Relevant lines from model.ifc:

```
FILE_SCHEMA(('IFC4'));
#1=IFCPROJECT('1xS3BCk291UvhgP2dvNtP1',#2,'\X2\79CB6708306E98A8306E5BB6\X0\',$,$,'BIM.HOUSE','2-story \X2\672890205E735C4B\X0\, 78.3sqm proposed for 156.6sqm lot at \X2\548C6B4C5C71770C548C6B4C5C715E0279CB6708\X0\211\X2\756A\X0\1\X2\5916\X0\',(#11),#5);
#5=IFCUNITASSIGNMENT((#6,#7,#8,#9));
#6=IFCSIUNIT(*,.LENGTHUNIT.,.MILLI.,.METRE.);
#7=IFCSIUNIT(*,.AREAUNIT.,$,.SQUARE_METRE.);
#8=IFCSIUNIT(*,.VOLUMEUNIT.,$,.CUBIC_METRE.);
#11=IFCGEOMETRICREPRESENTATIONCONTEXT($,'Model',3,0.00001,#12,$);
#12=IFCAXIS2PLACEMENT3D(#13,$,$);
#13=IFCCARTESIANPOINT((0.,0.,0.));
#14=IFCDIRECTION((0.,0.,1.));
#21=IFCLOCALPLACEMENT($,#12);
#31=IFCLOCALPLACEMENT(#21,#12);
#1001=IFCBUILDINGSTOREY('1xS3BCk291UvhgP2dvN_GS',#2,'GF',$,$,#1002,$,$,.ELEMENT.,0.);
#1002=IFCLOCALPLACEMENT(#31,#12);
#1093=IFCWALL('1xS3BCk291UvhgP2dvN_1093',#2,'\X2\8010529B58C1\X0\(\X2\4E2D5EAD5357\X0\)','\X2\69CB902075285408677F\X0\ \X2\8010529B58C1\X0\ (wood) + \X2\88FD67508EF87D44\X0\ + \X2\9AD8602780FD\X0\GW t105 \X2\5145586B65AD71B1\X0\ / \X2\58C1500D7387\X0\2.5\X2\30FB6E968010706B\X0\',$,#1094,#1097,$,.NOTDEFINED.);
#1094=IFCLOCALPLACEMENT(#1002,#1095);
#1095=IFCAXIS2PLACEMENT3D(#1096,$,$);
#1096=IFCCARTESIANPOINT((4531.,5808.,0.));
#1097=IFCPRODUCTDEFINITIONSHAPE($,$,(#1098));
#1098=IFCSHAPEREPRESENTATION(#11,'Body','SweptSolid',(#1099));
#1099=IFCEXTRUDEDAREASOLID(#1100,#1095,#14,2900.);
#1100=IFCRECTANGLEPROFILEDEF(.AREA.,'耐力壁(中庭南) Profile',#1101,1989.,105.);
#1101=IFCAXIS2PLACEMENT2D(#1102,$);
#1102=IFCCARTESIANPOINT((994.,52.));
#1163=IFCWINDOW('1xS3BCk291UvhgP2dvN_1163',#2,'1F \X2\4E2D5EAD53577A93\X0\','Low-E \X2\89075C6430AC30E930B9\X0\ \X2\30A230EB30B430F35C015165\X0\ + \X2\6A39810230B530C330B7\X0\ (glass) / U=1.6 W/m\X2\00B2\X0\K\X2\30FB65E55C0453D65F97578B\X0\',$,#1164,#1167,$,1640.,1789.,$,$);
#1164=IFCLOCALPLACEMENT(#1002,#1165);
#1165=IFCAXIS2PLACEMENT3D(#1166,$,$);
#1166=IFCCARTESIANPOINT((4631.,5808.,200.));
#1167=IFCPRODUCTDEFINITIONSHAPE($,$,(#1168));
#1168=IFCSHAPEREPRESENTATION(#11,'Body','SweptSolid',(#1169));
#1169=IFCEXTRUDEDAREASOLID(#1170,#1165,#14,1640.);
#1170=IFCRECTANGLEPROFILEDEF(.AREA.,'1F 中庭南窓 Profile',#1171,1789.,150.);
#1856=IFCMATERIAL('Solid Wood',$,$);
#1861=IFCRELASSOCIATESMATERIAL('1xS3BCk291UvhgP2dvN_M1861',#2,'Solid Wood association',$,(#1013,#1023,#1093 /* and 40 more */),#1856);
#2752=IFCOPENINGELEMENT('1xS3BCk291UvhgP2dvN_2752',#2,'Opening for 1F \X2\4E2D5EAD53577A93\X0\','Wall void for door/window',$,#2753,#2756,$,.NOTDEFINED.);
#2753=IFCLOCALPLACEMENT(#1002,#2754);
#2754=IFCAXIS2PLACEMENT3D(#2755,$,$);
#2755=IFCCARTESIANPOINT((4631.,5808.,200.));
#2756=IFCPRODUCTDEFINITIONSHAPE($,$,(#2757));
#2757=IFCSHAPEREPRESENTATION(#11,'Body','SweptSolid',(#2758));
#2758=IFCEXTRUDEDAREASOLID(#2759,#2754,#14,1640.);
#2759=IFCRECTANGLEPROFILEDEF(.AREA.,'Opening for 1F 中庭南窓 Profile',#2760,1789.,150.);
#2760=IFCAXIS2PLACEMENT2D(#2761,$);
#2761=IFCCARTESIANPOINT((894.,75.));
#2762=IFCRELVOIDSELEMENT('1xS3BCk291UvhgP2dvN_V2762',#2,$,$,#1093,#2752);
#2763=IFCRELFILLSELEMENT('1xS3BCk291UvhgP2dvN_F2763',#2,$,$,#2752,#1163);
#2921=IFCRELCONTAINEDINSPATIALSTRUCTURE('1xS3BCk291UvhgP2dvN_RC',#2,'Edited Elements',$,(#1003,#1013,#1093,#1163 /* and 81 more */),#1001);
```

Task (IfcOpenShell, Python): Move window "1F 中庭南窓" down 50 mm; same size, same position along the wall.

```python
import numpy as np
import ifcopenshell
import ifcopenshell.api.geometry
import ifcopenshell.util.placement
import ifcopenshell.util.unit

model = ifcopenshell.open("model.ifc")
unit_scale = ifcopenshell.util.unit.calculate_unit_scale(model)

window = model.by_guid("1xS3BCk291UvhgP2dvN_1163")
opening = window.FillsVoids[0].RelatingOpeningElement
dz = -50.0

shift = np.array([0.0, 0.0, dz])
# The window is not placed relative to its opening, so move both.
for product in (opening, window):
    matrix = ifcopenshell.util.placement.get_local_placement(product.ObjectPlacement)
    matrix[:3, 3] += shift
    ifcopenshell.api.geometry.edit_object_placement(model, product=product, matrix=matrix, is_si=False)

print(f"moved by {dz * unit_scale:+.3f} m")

model.write("model_updated.ifc")
```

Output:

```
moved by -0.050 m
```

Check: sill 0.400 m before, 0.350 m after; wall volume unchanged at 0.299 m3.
